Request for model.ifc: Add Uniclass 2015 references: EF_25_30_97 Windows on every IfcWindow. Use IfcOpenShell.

First a look at what the model holds.

```python
import ifcopenshell

model = ifcopenshell.open("model.ifc")
print(model.schema)
print("classifications:", [c.Name for c in model.by_type("IfcClassification")])
for ifc_class in ("IfcDoor", "IfcRoof", "IfcStair", "IfcWall", "IfcWindow"):
    print(ifc_class, len(model.by_type(ifc_class)))
```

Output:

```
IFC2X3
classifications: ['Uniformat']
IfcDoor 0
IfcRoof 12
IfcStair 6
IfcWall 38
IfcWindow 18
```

```python
import ifcopenshell
import ifcopenshell.api.classification

model = ifcopenshell.open("model.ifc")

# IFC2X3 requires Source and Edition and has no link from the project to the system.
system = model.create_entity("IfcClassification", Source="NBS", Edition="2015", Name="Uniclass 2015")

codes = {
    "IfcWindow": ("EF_25_30_97", "Windows"),
}
for ifc_class, (code, name) in codes.items():
    products = model.by_type(ifc_class)
    ifcopenshell.api.classification.add_reference(
        model, products=products, classification=system, identification=code, name=name
    )
    print(code, len(products))

model.write("model_rev.ifc")
```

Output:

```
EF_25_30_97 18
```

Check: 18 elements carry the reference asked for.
